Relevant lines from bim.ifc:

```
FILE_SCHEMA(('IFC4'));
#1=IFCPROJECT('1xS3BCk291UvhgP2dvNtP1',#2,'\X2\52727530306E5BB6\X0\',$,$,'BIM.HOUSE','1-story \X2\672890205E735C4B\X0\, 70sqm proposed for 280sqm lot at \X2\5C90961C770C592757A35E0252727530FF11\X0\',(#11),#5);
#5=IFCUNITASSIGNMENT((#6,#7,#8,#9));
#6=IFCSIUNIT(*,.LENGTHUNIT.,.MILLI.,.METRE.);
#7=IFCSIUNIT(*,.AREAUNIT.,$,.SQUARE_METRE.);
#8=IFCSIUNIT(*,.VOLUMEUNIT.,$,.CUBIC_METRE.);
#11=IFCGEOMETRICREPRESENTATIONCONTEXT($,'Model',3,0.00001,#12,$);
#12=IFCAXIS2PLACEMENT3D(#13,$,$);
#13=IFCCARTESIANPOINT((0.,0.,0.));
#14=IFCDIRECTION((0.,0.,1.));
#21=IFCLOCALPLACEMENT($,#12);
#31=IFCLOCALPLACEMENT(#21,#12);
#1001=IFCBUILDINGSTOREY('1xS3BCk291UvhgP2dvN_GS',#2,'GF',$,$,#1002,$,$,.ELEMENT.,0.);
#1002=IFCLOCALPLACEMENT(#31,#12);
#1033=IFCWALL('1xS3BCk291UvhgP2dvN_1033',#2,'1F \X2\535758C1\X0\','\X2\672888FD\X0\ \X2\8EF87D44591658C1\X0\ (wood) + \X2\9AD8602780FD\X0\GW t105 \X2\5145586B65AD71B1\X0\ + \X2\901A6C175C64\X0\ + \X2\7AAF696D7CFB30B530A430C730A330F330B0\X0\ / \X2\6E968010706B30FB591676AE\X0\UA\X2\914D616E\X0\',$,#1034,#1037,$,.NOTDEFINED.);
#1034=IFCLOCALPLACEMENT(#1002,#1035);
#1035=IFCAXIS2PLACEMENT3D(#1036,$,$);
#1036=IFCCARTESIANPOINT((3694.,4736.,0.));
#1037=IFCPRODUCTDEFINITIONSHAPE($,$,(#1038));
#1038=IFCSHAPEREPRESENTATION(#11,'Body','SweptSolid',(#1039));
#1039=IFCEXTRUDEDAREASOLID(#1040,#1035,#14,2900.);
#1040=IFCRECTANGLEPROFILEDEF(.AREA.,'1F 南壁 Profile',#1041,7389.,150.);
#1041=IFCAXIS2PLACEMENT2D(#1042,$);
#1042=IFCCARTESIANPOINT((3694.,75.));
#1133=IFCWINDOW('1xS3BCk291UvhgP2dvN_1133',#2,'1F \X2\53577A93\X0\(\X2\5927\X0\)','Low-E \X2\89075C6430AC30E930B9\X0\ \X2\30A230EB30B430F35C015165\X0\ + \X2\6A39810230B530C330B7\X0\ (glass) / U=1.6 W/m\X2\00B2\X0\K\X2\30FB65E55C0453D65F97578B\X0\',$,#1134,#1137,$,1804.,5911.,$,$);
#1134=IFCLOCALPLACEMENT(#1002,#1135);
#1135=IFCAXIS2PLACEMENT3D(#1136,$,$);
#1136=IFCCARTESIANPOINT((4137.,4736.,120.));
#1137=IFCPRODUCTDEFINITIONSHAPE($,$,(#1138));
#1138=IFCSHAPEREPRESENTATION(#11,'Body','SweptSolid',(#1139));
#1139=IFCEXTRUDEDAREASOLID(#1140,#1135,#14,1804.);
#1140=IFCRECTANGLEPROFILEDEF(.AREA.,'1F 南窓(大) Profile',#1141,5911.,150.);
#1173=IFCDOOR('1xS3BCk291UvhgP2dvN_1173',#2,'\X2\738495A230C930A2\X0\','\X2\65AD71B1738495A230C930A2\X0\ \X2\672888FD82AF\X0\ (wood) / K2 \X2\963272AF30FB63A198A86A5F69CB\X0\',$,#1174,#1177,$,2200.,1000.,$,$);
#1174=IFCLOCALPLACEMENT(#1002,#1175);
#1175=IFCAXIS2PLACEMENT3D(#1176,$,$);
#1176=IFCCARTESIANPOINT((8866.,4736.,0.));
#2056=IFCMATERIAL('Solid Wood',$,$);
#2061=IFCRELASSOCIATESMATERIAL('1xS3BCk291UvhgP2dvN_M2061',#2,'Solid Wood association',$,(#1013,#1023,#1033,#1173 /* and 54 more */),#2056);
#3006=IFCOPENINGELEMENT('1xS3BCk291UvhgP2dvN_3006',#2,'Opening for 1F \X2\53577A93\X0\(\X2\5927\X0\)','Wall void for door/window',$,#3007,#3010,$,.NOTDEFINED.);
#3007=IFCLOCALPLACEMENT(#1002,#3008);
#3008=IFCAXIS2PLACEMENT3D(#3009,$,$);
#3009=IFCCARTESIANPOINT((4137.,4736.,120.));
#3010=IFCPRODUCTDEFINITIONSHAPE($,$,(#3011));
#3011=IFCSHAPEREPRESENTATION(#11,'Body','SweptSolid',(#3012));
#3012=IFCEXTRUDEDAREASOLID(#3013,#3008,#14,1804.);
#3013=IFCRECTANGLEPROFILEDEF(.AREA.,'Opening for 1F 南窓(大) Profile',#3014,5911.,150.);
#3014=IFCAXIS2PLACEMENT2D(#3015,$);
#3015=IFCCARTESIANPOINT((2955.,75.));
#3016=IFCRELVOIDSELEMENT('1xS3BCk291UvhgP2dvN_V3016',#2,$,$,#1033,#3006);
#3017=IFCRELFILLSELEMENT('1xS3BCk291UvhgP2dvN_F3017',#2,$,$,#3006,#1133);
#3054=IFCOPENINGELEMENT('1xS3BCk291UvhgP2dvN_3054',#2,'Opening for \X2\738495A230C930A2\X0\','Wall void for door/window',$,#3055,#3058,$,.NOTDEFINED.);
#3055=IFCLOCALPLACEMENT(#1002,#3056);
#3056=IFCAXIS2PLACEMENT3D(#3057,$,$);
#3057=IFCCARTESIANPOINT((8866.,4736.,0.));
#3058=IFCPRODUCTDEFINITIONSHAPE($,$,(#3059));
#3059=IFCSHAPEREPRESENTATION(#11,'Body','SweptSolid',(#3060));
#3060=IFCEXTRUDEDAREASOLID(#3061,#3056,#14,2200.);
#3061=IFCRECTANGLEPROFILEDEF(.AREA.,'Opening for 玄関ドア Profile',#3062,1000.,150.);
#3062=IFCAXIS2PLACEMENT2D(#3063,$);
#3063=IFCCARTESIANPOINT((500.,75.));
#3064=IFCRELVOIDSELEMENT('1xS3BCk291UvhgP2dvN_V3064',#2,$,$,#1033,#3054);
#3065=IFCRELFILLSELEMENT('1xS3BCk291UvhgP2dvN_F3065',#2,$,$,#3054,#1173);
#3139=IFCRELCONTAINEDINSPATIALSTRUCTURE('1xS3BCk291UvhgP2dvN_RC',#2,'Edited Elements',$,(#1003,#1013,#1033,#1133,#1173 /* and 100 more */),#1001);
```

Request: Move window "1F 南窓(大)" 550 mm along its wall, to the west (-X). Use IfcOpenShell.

```python
import ifcopenshell
import ifcopenshell.api.geometry
import ifcopenshell.util.placement
import ifcopenshell.util.unit

model = ifcopenshell.open("bim.ifc")
unit_scale = ifcopenshell.util.unit.calculate_unit_scale(model)

window = model.by_guid("1xS3BCk291UvhgP2dvN_1133")
opening = window.FillsVoids[0].RelatingOpeningElement
wall = opening.VoidsElements[0].RelatingBuildingElement

wall_matrix = ifcopenshell.util.placement.get_local_placement(wall.ObjectPlacement)
shift = wall_matrix[:3, 0] * -0.55 / unit_scale
before = ifcopenshell.util.placement.get_local_placement(window.ObjectPlacement)[:3, 3].copy()

# The window is not placed relative to its opening, so move both.
for product in (opening, window):
    matrix = ifcopenshell.util.placement.get_local_placement(product.ObjectPlacement)
    matrix[:3, 3] += shift
    ifcopenshell.api.geometry.edit_object_placement(model, product=product, matrix=matrix, is_si=False)

after = ifcopenshell.util.placement.get_local_placement(window.ObjectPlacement)[:3, 3]
print("window moved by", (after - before).round(3) + 0.0)

model.write("bim_updated.ifc")
```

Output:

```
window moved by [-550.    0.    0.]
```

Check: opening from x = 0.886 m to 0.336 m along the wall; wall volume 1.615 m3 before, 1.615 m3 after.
